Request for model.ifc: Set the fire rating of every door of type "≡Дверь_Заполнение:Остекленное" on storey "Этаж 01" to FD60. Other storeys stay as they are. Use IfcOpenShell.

First a look at what the model holds.

```python
import ifcopenshell
import ifcopenshell.util.element

model = ifcopenshell.open("model.ifc")
print(model.schema)
storey = next(s for s in model.by_type("IfcBuildingStorey") if s.Name == "Этаж 01")
doors = [e for e in ifcopenshell.util.element.get_decomposition(storey) if e.is_a("IfcDoor")]
seen = {}
for e in doors:
    element_type = ifcopenshell.util.element.get_type(e)
    key = (element_type.Name if element_type != e and element_type else None, ifcopenshell.util.element.get_pset(e, "Pset_DoorCommon", "FireRating"))
    seen[key] = seen.get(key, 0) + 1
for (name, value), count in sorted(seen.items(), key=str):
    print(count, "x", name, "|", value)
```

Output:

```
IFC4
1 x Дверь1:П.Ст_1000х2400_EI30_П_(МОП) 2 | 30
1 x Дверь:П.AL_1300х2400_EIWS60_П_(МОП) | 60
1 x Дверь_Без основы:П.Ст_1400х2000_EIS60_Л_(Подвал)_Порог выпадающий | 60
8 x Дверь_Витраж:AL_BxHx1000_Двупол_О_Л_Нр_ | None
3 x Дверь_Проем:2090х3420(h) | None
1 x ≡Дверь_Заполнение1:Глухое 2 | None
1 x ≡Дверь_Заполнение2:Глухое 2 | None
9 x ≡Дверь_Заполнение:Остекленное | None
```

```python
import ifcopenshell
import ifcopenshell.api.pset
import ifcopenshell.util.element

model = ifcopenshell.open("model.ifc")

storey = next(s for s in model.by_type("IfcBuildingStorey") if s.Name == "Этаж 01")
doors = [e for e in ifcopenshell.util.element.get_decomposition(storey) if e.is_a("IfcDoor")]

count = 0
for e in doors:
    element_type = ifcopenshell.util.element.get_type(e)
    if element_type in (None, e) or element_type.Name != "≡Дверь_Заполнение:Остекленное":
        continue
    # add_pset returns the element's existing set when there is one.
    pset = ifcopenshell.api.pset.add_pset(model, product=e, name="Pset_DoorCommon")
    ifcopenshell.api.pset.edit_pset(model, pset=pset, properties={"FireRating": "FD60"})
    count += 1

print(count, "doors updated")

model.write("model_edited.ifc")
```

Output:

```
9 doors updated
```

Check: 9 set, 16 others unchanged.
